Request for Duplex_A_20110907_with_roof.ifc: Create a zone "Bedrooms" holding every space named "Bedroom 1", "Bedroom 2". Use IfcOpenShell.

First a look at what the model holds.

```python
import ifcopenshell

model = ifcopenshell.open("Duplex_A_20110907_with_roof.ifc")
print(model.schema)
seen = {}
for space in model.by_type("IfcSpace"):
    seen[space.LongName] = seen.get(space.LongName, 0) + 1
for name, count in sorted(seen.items(), key=str):
    print(count, "x", name)
print("zones:", [z.Name for z in model.by_type("IfcZone")][:20])
```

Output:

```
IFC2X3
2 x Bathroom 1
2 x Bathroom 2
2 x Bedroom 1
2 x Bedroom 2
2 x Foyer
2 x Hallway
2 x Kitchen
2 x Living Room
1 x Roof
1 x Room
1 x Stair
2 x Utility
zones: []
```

```python
import ifcopenshell
import ifcopenshell.api.group
import ifcopenshell.api.root

model = ifcopenshell.open("Duplex_A_20110907_with_roof.ifc")

names = {"Bedroom 1", "Bedroom 2"}
spaces = [s for s in model.by_type("IfcSpace") if s.LongName in names]

zone = ifcopenshell.api.root.create_entity(model, ifc_class="IfcZone", name="Bedrooms")
ifcopenshell.api.group.assign_group(model, products=spaces, group=zone)
print(len(spaces), "spaces in", zone.Name)

model.write("Duplex_A_20110907_with_roof_rev.ifc")
```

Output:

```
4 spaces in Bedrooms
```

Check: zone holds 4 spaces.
